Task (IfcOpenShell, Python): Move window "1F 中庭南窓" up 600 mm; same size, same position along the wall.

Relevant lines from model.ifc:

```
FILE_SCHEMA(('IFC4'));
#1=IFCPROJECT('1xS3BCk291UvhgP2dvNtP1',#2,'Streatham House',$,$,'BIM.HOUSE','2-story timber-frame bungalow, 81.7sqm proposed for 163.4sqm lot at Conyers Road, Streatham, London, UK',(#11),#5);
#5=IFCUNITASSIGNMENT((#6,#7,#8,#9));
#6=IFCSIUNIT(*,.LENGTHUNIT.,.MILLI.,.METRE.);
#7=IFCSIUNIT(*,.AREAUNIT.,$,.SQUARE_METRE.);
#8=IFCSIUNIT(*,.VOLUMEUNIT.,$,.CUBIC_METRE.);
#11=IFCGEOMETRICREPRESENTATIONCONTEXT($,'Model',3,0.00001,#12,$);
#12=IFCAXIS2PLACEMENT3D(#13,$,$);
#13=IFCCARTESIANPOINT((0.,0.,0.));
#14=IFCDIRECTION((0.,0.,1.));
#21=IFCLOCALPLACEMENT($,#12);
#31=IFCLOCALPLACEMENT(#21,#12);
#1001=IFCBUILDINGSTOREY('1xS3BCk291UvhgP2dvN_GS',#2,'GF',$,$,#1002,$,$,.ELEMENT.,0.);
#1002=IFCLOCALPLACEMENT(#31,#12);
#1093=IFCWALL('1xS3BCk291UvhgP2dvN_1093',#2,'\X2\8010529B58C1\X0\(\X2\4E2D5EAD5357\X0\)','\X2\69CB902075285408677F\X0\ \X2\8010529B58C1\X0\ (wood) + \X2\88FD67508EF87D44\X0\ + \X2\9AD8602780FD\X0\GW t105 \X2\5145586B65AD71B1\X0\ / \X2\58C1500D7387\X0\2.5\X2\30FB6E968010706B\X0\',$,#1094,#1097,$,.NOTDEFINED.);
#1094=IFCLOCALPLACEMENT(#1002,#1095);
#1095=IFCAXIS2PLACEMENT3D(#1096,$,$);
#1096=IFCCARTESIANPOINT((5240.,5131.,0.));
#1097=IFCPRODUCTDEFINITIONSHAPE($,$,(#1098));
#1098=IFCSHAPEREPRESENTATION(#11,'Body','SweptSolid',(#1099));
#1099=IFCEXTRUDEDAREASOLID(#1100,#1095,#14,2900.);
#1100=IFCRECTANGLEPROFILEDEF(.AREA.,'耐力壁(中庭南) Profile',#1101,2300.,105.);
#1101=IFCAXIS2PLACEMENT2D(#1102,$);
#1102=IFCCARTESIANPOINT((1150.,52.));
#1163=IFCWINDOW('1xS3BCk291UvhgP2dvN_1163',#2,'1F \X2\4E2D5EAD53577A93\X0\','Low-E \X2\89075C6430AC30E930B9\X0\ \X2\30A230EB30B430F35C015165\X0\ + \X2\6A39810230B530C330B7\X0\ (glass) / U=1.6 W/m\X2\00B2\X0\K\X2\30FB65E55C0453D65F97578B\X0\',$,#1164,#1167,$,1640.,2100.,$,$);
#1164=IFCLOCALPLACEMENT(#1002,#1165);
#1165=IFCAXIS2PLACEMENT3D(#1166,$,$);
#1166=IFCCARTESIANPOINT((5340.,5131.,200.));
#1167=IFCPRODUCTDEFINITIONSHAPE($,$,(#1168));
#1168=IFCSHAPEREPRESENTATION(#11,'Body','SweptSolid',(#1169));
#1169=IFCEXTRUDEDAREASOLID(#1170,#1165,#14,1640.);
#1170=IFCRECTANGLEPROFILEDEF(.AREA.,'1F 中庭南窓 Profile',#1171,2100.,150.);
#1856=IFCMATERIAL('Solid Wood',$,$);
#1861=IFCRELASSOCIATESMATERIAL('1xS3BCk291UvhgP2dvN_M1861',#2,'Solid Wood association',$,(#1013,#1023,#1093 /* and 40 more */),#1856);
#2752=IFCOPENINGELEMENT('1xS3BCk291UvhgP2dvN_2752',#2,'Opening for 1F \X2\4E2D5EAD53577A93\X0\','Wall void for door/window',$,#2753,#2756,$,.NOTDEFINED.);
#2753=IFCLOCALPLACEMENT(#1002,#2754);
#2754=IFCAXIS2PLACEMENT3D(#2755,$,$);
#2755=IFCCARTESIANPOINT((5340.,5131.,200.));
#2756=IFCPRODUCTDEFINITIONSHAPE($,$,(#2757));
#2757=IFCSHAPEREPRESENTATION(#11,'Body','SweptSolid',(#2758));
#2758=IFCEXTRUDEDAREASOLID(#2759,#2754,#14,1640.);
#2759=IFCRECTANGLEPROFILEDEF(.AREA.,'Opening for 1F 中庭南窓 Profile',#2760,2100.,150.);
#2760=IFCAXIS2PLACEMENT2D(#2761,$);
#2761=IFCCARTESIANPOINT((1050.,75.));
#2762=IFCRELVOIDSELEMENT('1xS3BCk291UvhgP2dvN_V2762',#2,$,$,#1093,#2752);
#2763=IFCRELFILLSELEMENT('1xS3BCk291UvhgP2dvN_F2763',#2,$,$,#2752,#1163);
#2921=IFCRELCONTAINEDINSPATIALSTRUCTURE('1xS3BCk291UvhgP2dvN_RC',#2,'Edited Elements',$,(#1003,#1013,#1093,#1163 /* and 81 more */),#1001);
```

```python
import numpy as np
import ifcopenshell
import ifcopenshell.api.geometry
import ifcopenshell.util.placement
import ifcopenshell.util.unit

model = ifcopenshell.open("model.ifc")
unit_scale = ifcopenshell.util.unit.calculate_unit_scale(model)

window = model.by_id(1163)
opening = window.FillsVoids[0].RelatingOpeningElement
dz = 600.0

shift = np.array([0.0, 0.0, dz])
# The window is not placed relative to its opening, so move both.
for product in (opening, window):
    matrix = ifcopenshell.util.placement.get_local_placement(product.ObjectPlacement)
    matrix[:3, 3] += shift
    ifcopenshell.api.geometry.edit_object_placement(model, product=product, matrix=matrix, is_si=False)

print(f"moved by {dz * unit_scale:+.3f} m")

model.write("model_updated.ifc")
```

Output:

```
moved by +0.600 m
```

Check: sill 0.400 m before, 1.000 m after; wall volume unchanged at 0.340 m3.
